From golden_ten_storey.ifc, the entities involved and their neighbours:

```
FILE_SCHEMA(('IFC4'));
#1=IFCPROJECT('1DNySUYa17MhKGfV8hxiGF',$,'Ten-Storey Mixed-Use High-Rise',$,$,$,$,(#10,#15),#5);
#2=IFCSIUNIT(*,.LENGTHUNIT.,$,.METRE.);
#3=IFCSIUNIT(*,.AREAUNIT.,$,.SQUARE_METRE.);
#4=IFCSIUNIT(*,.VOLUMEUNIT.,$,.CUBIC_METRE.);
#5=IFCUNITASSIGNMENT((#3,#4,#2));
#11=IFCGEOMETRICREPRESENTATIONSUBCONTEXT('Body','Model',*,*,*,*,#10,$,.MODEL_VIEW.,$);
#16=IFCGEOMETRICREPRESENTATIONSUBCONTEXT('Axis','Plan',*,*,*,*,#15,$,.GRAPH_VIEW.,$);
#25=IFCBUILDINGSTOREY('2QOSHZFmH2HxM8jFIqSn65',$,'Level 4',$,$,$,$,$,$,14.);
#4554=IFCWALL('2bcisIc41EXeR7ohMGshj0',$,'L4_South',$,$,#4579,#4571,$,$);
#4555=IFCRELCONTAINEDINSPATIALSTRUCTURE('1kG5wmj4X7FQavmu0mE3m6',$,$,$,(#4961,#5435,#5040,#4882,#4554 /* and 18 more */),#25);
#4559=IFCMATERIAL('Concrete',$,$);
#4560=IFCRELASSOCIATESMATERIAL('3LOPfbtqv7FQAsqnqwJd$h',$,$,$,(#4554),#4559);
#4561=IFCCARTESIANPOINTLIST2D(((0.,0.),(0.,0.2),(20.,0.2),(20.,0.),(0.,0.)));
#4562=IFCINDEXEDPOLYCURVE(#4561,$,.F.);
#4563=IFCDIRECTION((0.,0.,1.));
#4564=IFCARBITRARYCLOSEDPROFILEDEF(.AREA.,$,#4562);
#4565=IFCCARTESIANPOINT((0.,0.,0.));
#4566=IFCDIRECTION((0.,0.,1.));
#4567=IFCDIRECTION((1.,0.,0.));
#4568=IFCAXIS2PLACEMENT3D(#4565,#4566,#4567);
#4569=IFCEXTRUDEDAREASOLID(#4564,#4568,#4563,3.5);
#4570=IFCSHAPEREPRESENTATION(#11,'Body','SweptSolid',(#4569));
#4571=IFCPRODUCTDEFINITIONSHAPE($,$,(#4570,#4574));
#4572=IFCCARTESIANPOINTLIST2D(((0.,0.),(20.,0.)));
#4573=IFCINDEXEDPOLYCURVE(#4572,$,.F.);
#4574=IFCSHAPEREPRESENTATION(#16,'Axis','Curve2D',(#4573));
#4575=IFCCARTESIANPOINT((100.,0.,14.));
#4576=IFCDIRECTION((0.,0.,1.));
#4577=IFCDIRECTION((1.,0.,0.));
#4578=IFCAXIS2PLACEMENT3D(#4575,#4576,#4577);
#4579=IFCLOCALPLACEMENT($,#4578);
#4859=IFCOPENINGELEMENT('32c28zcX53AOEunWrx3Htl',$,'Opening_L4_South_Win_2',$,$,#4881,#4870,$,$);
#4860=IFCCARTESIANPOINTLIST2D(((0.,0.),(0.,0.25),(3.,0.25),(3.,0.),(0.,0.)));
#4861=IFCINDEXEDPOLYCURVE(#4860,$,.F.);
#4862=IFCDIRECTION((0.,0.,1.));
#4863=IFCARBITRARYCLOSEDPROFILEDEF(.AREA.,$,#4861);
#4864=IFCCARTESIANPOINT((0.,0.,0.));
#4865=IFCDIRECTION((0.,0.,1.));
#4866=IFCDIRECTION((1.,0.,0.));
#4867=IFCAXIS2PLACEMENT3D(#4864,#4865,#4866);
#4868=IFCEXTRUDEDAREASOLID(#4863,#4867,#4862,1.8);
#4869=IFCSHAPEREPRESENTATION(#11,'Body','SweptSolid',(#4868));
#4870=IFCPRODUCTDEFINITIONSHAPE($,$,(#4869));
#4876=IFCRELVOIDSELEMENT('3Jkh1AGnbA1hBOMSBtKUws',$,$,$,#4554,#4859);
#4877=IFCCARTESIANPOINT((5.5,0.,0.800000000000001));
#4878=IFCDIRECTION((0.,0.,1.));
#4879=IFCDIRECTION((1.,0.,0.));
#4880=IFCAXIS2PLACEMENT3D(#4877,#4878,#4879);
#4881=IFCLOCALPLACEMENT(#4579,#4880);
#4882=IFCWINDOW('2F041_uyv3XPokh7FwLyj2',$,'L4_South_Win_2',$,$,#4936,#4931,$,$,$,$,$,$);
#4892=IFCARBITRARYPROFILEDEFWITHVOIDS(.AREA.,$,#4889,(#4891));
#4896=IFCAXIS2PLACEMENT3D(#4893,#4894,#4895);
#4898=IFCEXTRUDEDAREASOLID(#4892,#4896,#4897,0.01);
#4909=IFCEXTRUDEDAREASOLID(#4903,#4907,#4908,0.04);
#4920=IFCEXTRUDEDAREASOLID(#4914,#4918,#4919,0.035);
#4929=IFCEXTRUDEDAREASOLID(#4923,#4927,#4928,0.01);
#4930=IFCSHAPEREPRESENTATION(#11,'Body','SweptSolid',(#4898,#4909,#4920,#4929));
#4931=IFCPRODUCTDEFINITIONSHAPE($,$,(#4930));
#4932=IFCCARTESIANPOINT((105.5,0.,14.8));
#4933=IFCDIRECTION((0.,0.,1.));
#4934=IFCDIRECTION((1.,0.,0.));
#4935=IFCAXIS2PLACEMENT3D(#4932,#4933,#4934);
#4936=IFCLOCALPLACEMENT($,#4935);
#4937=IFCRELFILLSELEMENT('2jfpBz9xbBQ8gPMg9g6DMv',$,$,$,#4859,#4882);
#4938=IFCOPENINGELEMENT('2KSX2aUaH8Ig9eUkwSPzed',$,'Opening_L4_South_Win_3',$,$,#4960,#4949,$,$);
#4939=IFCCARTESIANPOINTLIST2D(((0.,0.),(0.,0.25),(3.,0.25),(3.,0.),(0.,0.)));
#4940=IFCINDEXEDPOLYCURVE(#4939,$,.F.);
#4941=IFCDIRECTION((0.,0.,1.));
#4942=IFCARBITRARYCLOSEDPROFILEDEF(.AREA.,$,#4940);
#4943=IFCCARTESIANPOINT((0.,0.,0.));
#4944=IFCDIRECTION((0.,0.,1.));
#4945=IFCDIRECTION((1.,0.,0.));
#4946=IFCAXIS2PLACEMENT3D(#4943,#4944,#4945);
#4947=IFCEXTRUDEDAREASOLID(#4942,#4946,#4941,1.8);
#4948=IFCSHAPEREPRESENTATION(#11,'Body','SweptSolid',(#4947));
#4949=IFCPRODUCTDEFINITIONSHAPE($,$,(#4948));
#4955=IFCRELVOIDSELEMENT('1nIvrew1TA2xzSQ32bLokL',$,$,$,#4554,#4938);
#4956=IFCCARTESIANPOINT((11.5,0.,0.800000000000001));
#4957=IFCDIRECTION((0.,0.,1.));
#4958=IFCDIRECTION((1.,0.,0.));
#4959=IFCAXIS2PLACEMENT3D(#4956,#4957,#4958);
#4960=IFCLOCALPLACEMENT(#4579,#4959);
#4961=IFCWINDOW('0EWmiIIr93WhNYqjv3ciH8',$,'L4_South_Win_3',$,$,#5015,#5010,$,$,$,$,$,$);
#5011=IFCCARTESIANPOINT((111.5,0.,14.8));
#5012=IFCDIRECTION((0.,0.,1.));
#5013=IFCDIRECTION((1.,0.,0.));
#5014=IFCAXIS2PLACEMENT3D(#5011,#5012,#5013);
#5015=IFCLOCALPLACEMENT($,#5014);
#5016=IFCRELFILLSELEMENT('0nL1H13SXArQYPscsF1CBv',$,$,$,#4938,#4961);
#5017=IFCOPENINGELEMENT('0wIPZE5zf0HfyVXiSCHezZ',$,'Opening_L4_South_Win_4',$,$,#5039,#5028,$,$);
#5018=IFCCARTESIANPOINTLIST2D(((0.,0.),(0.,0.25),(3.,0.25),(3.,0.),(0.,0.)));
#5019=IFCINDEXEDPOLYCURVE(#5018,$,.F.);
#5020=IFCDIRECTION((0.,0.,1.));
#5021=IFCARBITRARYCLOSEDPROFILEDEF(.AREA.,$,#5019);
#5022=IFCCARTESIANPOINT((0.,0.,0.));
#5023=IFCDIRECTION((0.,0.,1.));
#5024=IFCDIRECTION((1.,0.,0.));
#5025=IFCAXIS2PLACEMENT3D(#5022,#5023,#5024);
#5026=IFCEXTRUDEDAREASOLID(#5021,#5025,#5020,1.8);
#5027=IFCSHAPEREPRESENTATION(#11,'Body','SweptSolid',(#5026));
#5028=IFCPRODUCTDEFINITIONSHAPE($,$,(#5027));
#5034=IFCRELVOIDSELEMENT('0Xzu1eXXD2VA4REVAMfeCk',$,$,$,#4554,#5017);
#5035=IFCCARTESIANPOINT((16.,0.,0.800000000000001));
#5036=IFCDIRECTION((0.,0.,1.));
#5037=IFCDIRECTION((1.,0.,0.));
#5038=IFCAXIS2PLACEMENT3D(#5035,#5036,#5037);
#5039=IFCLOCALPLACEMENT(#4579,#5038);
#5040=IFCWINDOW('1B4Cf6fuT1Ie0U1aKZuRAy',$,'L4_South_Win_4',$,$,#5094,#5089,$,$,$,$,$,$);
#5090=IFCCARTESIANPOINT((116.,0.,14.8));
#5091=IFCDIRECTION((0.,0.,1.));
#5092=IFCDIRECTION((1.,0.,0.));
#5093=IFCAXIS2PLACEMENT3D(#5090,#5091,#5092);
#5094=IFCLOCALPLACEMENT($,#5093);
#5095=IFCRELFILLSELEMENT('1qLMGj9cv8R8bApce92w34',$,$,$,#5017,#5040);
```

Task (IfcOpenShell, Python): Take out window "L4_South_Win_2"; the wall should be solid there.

```python
import ifcopenshell
import ifcopenshell.api.feature
import ifcopenshell.api.root
import ifcopenshell.geom
import ifcopenshell.util.shape

model = ifcopenshell.open("golden_ten_storey.ifc")
settings = ifcopenshell.geom.settings()


def volume(element):
    """Net volume in cubic metres, openings subtracted."""
    shape = ifcopenshell.geom.create_shape(settings, element)
    return ifcopenshell.util.shape.get_volume(shape.geometry)


window = model.by_guid("2F041_uyv3XPokh7FwLyj2")
opening = window.FillsVoids[0].RelatingOpeningElement
wall = opening.VoidsElements[0].RelatingBuildingElement
before = volume(wall)

ifcopenshell.api.root.remove_product(model, product=window)
ifcopenshell.api.feature.remove_feature(model, feature=opening)

after = volume(wall)

print(f"wall volume {before:.3f} -> {after:.3f} m3")

model.write("golden_ten_storey_updated.ifc")
```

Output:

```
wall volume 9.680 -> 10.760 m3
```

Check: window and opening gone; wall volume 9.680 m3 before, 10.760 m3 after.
